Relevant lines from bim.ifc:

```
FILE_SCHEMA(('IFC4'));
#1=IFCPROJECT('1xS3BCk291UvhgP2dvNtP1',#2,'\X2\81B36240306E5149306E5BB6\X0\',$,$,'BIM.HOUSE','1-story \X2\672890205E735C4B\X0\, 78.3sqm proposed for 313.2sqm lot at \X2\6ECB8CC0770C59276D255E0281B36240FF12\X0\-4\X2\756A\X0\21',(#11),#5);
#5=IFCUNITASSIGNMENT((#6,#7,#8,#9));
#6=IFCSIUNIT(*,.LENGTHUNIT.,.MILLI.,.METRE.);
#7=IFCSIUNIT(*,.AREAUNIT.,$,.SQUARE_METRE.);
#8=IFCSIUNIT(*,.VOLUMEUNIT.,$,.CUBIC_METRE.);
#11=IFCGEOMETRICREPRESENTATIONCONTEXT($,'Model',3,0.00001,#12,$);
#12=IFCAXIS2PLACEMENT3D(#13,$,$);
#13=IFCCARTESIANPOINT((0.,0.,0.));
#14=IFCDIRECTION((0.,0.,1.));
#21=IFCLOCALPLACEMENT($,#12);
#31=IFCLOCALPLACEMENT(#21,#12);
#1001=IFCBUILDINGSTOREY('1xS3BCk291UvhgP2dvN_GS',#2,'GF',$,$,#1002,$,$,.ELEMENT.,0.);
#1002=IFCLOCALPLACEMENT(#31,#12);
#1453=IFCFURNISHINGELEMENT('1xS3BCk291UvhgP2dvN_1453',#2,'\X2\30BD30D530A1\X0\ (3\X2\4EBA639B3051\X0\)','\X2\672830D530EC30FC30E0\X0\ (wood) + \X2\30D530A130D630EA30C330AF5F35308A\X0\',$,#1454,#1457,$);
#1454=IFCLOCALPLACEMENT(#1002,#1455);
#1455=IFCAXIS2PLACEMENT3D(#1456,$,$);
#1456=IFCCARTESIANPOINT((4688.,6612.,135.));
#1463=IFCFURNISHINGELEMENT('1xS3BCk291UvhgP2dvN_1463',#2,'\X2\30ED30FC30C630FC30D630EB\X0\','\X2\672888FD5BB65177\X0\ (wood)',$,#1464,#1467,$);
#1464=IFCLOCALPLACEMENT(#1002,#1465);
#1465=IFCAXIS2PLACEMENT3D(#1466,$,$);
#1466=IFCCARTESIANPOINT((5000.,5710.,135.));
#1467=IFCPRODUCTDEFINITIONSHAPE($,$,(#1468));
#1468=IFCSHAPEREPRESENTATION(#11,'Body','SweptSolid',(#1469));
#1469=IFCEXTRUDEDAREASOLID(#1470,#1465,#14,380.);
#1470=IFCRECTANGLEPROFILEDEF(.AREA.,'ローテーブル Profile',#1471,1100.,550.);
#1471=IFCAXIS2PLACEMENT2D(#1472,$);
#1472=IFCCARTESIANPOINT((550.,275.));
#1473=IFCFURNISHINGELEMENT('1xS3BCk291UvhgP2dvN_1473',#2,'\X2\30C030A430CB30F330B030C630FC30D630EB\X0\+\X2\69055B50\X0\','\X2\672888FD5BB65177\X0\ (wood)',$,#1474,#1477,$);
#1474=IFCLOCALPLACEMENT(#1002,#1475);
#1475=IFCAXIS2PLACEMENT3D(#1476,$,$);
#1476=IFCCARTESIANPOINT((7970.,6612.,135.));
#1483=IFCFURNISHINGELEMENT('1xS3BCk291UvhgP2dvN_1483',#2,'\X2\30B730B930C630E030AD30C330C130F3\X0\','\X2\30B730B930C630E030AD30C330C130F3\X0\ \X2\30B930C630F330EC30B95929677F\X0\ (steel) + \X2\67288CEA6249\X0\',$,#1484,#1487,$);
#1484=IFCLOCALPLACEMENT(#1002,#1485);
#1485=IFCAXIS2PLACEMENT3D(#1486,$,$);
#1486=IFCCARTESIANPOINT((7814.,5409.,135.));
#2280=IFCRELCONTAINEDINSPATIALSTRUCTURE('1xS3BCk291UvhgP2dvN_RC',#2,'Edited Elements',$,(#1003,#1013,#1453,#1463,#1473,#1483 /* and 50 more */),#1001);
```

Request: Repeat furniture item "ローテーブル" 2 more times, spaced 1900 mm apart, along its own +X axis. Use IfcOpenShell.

```python
import ifcopenshell
import ifcopenshell.api.geometry
import ifcopenshell.api.root
import ifcopenshell.util.element
import ifcopenshell.util.placement
import ifcopenshell.util.unit

model = ifcopenshell.open("bim.ifc")
unit_scale = ifcopenshell.util.unit.calculate_unit_scale(model)


def reuse_history(source, copy):
    """copy_class also copies each property set's owner history, people and application; keep the originals."""
    for rel in copy.IsDefinedBy:
        if rel.is_a("IfcRelDefinesByProperties") and (history := rel.RelatingPropertyDefinition.OwnerHistory):
            rel.RelatingPropertyDefinition.OwnerHistory = source.OwnerHistory
            ifcopenshell.util.element.remove_deep2(model, history)


source = model.by_guid("1xS3BCk291UvhgP2dvN_1463")
base = ifcopenshell.util.placement.get_local_placement(source.ObjectPlacement)
step = base[:3, 0] * 1.9 / unit_scale

for i in range(1, 3):
    copy = ifcopenshell.api.root.copy_class(model, product=source)
    copy.Representation = ifcopenshell.util.element.copy_deep(
        model, source.Representation, exclude=["IfcGeometricRepresentationContext", "IfcRepresentationMap"]
    )
    reuse_history(source, copy)
    matrix = base.copy()
    matrix[:3, 3] += i * step
    print("added at", matrix[:3, 3].round(3) + 0.0)
    ifcopenshell.api.geometry.edit_object_placement(model, product=copy, matrix=matrix, is_si=False)

model.write("bim_rev.ifc")
```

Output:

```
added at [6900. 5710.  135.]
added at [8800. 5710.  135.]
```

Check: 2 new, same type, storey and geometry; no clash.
